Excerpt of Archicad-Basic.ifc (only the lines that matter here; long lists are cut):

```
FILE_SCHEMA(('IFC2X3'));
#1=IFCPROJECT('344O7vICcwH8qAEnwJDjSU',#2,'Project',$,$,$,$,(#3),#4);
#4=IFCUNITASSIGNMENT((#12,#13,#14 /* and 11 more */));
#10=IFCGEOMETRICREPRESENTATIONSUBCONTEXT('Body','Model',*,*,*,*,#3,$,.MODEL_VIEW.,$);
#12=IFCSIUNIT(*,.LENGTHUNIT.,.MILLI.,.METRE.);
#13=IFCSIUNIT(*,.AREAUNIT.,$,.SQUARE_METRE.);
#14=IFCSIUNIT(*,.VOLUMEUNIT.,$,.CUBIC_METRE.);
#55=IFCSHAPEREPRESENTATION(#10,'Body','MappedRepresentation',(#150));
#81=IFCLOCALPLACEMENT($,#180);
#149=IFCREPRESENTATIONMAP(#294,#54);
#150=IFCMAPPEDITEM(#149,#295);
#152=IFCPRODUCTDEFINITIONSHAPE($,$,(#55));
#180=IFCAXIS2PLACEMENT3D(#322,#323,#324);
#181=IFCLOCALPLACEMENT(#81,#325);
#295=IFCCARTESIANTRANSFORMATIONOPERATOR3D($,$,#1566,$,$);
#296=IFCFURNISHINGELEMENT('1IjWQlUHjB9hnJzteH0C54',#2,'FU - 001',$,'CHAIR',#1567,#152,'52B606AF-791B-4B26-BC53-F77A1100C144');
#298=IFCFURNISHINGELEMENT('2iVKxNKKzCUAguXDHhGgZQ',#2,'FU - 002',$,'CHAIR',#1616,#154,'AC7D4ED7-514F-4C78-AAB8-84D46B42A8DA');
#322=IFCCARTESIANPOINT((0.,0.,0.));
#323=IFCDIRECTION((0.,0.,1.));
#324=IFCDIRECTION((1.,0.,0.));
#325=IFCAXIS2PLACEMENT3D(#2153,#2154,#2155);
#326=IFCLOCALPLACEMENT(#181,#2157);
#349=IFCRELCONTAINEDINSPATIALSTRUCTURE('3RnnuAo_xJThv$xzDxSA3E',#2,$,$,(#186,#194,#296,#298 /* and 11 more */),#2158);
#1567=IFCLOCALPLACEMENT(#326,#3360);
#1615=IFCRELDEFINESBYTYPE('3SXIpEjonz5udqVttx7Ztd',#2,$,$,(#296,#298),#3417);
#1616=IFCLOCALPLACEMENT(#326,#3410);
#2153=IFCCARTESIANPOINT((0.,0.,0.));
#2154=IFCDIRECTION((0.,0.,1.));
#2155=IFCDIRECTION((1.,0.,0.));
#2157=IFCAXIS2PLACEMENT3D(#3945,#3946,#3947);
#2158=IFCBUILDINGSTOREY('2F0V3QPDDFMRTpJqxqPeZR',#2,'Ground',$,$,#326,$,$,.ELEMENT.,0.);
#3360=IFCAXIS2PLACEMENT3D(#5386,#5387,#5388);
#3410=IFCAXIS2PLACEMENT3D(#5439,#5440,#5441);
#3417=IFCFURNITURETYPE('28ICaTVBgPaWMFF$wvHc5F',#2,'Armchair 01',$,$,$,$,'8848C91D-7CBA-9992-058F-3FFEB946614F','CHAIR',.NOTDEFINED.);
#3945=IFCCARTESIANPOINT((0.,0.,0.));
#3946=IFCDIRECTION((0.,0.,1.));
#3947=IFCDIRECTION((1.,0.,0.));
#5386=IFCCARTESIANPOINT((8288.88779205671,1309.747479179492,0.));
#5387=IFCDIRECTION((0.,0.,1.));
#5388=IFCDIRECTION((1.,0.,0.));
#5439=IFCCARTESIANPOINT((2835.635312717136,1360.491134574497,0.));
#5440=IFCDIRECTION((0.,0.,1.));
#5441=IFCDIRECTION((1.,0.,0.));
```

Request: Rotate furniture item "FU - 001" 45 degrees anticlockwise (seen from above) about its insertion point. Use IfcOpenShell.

```python
import ifcopenshell
import ifcopenshell.api.geometry
import ifcopenshell.util.placement

model = ifcopenshell.open("Archicad-Basic.ifc")

item = model.by_id(296)
matrix = ifcopenshell.util.placement.get_local_placement(item.ObjectPlacement)
matrix = matrix @ ifcopenshell.util.placement.rotation(45, "Z")
ifcopenshell.api.geometry.edit_object_placement(model, product=item, matrix=matrix, is_si=False)

print(ifcopenshell.util.placement.get_local_placement(item.ObjectPlacement).round(3) + 0.0)

model.write("Archicad-Basic-out.ifc")
```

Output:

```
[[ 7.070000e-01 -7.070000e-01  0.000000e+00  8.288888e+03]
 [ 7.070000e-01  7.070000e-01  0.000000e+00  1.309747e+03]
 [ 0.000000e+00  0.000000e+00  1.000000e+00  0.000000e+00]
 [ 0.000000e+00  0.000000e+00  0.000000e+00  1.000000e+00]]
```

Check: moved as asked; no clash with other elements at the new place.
